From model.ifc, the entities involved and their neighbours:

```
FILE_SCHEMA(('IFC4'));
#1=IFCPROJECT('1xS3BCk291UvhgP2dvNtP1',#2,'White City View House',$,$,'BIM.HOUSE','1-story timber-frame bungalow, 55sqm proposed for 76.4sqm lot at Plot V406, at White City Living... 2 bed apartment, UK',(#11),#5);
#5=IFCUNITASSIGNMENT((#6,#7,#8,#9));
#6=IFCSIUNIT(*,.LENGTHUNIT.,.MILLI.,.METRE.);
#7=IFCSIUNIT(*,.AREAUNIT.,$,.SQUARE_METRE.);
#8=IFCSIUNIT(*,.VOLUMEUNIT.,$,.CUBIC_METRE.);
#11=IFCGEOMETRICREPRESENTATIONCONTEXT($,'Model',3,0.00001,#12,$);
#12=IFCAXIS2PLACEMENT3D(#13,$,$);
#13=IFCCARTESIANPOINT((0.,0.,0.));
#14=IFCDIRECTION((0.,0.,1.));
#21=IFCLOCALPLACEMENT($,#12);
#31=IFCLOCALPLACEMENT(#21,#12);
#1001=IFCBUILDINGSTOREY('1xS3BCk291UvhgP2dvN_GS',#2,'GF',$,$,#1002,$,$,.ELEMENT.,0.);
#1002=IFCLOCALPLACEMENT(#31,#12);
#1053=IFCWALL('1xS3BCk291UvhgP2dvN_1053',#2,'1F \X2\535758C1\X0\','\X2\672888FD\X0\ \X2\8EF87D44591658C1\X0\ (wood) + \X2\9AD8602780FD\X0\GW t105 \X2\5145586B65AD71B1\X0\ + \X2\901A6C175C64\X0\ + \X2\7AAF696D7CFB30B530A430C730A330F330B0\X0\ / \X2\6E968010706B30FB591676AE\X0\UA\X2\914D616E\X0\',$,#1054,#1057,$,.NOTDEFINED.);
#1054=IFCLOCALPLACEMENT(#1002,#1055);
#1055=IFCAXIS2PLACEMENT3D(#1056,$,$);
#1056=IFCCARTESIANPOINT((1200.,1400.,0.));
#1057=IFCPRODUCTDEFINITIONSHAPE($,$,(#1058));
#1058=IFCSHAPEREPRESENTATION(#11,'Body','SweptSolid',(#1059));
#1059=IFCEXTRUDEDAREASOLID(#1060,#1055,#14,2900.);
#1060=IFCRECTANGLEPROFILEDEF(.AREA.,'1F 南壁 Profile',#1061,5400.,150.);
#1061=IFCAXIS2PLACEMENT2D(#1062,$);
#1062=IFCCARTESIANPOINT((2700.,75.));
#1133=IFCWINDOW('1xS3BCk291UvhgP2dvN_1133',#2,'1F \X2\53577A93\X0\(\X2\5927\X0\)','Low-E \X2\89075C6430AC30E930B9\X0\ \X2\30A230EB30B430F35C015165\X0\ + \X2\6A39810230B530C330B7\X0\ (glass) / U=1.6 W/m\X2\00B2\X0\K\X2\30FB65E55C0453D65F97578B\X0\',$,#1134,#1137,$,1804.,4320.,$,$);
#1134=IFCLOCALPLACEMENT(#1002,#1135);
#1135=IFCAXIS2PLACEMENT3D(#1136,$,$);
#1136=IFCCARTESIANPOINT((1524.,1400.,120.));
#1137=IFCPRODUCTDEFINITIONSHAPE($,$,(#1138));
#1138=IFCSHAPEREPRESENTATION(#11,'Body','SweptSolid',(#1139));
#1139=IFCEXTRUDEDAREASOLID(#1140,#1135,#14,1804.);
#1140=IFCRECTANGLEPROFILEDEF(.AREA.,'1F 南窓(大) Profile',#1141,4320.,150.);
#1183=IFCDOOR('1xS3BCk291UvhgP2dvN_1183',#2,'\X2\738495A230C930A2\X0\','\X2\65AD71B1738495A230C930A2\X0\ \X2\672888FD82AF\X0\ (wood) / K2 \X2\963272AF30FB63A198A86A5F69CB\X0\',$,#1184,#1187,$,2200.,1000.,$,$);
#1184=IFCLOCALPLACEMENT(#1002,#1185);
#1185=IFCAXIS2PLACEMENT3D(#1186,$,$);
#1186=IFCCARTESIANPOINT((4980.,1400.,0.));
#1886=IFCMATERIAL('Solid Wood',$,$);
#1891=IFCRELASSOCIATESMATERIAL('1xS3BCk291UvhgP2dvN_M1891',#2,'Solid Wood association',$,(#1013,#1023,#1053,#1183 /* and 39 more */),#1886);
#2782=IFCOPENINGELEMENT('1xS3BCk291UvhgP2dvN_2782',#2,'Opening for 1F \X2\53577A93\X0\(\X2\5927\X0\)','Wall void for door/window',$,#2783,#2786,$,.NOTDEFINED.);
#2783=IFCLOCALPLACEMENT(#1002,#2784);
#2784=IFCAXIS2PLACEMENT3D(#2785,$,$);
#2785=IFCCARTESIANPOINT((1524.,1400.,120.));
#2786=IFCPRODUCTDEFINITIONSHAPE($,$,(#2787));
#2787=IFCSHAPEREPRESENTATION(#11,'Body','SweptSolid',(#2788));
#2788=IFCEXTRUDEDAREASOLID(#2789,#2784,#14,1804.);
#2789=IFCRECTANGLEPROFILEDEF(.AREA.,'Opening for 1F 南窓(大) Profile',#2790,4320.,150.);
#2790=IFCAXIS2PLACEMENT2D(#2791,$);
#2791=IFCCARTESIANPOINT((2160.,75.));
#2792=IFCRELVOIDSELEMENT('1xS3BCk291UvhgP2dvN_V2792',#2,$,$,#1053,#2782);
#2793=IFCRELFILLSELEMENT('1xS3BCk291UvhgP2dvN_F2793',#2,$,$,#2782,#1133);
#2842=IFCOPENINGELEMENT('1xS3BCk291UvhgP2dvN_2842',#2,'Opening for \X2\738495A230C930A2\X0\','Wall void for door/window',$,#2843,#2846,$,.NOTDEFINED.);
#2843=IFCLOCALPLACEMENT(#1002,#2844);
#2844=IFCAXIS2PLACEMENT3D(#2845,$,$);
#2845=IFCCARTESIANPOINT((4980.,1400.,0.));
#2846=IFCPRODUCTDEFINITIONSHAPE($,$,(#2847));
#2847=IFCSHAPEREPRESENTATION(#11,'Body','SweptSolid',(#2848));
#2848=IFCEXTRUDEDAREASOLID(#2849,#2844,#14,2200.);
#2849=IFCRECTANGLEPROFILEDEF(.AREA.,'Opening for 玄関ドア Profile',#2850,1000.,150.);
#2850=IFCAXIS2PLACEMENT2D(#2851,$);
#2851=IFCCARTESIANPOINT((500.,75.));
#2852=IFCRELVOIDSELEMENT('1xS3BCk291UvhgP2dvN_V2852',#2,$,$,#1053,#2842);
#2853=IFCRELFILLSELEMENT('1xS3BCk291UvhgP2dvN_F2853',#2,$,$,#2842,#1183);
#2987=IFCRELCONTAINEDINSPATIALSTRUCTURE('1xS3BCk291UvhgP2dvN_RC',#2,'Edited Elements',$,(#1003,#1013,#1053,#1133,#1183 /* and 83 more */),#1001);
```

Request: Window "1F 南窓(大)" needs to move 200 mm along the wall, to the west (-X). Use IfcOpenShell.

```python
import ifcopenshell
import ifcopenshell.api.geometry
import ifcopenshell.util.placement

model = ifcopenshell.open("model.ifc")

window = model.by_id(1133)
opening = window.FillsVoids[0].RelatingOpeningElement
wall = opening.VoidsElements[0].RelatingBuildingElement

wall_matrix = ifcopenshell.util.placement.get_local_placement(wall.ObjectPlacement)
shift = wall_matrix[:3, 0] * -200.0
before = ifcopenshell.util.placement.get_local_placement(window.ObjectPlacement)[:3, 3].copy()

# The window is not placed relative to its opening, so move both.
for product in (opening, window):
    matrix = ifcopenshell.util.placement.get_local_placement(product.ObjectPlacement)
    matrix[:3, 3] += shift
    ifcopenshell.api.geometry.edit_object_placement(model, product=product, matrix=matrix, is_si=False)

after = ifcopenshell.util.placement.get_local_placement(window.ObjectPlacement)[:3, 3]
print("window moved by", (after - before).round(3) + 0.0)

model.write("model_rev.ifc")
```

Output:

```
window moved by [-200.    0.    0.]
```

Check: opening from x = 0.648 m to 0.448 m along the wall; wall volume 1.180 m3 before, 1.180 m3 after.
